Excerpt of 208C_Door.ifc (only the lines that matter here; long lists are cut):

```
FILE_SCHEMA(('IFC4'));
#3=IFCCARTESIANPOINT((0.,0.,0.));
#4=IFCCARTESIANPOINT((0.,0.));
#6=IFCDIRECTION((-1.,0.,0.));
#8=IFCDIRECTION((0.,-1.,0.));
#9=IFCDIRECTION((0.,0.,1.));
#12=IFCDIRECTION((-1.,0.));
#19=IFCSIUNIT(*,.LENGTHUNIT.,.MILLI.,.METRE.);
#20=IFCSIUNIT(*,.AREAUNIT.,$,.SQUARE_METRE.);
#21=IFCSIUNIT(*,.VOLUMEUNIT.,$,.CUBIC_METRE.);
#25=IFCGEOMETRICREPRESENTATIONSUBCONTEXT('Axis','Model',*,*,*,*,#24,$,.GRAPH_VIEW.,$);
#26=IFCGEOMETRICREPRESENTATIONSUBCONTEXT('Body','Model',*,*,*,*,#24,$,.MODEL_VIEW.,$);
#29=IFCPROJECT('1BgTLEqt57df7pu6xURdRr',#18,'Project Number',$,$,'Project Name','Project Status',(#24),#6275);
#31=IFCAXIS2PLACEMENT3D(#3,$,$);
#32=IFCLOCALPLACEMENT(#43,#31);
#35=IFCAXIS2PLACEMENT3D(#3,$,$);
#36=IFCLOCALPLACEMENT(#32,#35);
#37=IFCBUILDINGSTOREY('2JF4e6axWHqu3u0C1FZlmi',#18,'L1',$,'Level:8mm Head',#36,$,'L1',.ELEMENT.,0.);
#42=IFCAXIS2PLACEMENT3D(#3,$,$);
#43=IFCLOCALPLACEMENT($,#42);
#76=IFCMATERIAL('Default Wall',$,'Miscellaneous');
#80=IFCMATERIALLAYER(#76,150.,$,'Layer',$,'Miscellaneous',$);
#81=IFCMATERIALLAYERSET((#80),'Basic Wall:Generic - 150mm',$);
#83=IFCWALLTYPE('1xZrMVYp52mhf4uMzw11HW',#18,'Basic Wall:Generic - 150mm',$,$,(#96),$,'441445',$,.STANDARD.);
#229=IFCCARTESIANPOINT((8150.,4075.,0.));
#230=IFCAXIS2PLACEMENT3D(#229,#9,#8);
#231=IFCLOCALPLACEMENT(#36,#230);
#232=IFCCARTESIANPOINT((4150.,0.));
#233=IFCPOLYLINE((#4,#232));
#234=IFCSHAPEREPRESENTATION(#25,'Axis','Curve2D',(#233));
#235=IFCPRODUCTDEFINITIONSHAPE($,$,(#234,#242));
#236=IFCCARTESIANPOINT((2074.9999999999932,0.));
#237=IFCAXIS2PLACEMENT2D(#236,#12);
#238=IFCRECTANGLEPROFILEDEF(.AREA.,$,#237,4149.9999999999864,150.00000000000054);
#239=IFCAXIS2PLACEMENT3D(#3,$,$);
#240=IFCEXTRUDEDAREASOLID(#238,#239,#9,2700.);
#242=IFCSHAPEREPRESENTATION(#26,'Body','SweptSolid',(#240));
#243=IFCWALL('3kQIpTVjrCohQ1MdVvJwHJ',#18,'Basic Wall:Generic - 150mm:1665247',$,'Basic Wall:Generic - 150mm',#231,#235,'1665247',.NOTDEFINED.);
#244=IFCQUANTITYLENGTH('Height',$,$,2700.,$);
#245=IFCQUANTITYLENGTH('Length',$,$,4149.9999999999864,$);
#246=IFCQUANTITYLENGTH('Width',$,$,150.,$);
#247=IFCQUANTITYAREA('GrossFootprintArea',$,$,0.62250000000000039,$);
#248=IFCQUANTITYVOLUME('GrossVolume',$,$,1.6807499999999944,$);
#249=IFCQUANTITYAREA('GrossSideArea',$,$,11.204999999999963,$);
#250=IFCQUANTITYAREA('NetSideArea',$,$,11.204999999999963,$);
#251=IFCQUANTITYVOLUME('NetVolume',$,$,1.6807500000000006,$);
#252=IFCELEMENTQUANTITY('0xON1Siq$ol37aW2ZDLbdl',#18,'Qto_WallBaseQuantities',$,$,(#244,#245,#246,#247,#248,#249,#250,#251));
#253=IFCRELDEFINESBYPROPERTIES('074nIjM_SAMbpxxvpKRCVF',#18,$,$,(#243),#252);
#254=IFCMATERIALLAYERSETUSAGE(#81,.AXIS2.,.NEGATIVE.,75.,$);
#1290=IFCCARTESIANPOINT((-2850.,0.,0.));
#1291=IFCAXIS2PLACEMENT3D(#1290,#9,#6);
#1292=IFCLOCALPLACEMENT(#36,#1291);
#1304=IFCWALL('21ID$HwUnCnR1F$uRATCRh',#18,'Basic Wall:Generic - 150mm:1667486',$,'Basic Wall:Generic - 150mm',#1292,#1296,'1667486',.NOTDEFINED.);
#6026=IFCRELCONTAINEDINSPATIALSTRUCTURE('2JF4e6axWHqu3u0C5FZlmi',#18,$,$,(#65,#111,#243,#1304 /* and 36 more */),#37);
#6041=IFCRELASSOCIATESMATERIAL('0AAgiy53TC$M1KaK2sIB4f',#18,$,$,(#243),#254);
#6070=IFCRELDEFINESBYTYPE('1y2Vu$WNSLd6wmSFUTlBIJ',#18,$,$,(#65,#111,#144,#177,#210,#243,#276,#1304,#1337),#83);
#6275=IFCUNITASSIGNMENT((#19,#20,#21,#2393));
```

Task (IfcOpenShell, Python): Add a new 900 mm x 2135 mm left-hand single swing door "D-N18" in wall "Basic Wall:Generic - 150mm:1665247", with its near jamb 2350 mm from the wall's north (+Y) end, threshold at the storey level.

```python
import numpy as np
import ifcopenshell
import ifcopenshell.api.feature
import ifcopenshell.api.geometry
import ifcopenshell.api.pset
import ifcopenshell.api.root
import ifcopenshell.api.spatial
import ifcopenshell.geom
import ifcopenshell.util.element
import ifcopenshell.util.placement
import ifcopenshell.util.representation
import ifcopenshell.util.shape
import ifcopenshell.util.unit

model = ifcopenshell.open("208C_Door.ifc")
unit_scale = ifcopenshell.util.unit.calculate_unit_scale(model)
area_scale = ifcopenshell.util.unit.calculate_unit_scale(model, "AREAUNIT")
volume_scale = ifcopenshell.util.unit.calculate_unit_scale(model, "VOLUMEUNIT")
settings = ifcopenshell.geom.settings()


def volume(element):
    """Net volume in cubic metres, openings subtracted."""
    shape = ifcopenshell.geom.create_shape(settings, element)
    return ifcopenshell.util.shape.get_volume(shape.geometry)


wall = model.by_guid("3kQIpTVjrCohQ1MdVvJwHJ")
storey = ifcopenshell.util.element.get_container(wall, ifc_class="IfcBuildingStorey")
context = ifcopenshell.util.representation.get_context(model, "Model", "Body", "MODEL_VIEW")
before = volume(wall)

width, height, from_end, sill = 0.9, 2.135, 2.35, 0.0  # metres

# The wall runs along its own X axis, and the end named is its -X end.
wall_shape = ifcopenshell.geom.create_shape(settings, wall)
x, y, z = ifcopenshell.util.shape.get_vertices(wall_shape.geometry).T
start = x.min() + from_end
face, thickness = float(y.min()), float(y.max() - y.min())
wall_matrix = ifcopenshell.util.placement.get_local_placement(wall.ObjectPlacement)
level = ifcopenshell.util.placement.get_local_placement(storey.ObjectPlacement)[2, 3]


def in_wall(x, y):
    """Placement at x, y metres in the wall's axes, at sill height."""
    matrix = wall_matrix.copy()
    matrix[:, 3] = wall_matrix @ np.array([x / unit_scale, y / unit_scale, 0.0, 1.0])
    matrix[2, 3] = level + sill / unit_scale
    return matrix


# Opening: a box that overshoots both wall faces by 50 mm.
opening = ifcopenshell.api.root.create_entity(model, ifc_class="IfcOpeningElement", predefined_type="OPENING")
box = ifcopenshell.api.geometry.add_wall_representation(
    model, context=context, length=width, height=height, thickness=thickness + 0.1
)
ifcopenshell.api.geometry.assign_representation(model, product=opening, representation=box)
ifcopenshell.api.geometry.edit_object_placement(model, product=opening, matrix=in_wall(start, face - 0.05), is_si=False)
ifcopenshell.api.feature.add_feature(model, feature=opening, element=wall)

door = ifcopenshell.api.root.create_entity(model, ifc_class="IfcDoor", name="D-N18", predefined_type="DOOR")
door.OverallWidth, door.OverallHeight = width / unit_scale, height / unit_scale
door.OperationType = "SINGLE_SWING_LEFT"
body = ifcopenshell.api.geometry.add_door_representation(
    model,
    context=context,
    overall_width=door.OverallWidth,
    overall_height=door.OverallHeight,
    operation_type="SINGLE_SWING_LEFT",
    lining_properties={"LiningDepth": thickness / unit_scale, "ThresholdDepth": thickness / unit_scale},
)
ifcopenshell.api.geometry.assign_representation(model, product=door, representation=body)
ifcopenshell.api.spatial.assign_container(model, products=[door], relating_structure=storey)
ifcopenshell.api.feature.add_filling(model, opening=opening, element=door)

# The lining spans the wall, so the door starts at the wall face.
ifcopenshell.api.geometry.edit_object_placement(model, product=door, matrix=in_wall(start, face), is_si=False)

after = volume(wall)

# Update the wall's stored quantities.
qto = model.by_id(ifcopenshell.util.element.get_pset(wall, "Qto_WallBaseQuantities", should_inherit=False)["id"])
ifcopenshell.api.pset.edit_qto(model, qto=qto, properties={
    "NetSideArea": after / thickness / area_scale,
    "NetVolume": after / volume_scale,
})

print(f"wall volume {before:.3f} -> {after:.3f} m3")

model.write("208C_Door_edited.ifc")
```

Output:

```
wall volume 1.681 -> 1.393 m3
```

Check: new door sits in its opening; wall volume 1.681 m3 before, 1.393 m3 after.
